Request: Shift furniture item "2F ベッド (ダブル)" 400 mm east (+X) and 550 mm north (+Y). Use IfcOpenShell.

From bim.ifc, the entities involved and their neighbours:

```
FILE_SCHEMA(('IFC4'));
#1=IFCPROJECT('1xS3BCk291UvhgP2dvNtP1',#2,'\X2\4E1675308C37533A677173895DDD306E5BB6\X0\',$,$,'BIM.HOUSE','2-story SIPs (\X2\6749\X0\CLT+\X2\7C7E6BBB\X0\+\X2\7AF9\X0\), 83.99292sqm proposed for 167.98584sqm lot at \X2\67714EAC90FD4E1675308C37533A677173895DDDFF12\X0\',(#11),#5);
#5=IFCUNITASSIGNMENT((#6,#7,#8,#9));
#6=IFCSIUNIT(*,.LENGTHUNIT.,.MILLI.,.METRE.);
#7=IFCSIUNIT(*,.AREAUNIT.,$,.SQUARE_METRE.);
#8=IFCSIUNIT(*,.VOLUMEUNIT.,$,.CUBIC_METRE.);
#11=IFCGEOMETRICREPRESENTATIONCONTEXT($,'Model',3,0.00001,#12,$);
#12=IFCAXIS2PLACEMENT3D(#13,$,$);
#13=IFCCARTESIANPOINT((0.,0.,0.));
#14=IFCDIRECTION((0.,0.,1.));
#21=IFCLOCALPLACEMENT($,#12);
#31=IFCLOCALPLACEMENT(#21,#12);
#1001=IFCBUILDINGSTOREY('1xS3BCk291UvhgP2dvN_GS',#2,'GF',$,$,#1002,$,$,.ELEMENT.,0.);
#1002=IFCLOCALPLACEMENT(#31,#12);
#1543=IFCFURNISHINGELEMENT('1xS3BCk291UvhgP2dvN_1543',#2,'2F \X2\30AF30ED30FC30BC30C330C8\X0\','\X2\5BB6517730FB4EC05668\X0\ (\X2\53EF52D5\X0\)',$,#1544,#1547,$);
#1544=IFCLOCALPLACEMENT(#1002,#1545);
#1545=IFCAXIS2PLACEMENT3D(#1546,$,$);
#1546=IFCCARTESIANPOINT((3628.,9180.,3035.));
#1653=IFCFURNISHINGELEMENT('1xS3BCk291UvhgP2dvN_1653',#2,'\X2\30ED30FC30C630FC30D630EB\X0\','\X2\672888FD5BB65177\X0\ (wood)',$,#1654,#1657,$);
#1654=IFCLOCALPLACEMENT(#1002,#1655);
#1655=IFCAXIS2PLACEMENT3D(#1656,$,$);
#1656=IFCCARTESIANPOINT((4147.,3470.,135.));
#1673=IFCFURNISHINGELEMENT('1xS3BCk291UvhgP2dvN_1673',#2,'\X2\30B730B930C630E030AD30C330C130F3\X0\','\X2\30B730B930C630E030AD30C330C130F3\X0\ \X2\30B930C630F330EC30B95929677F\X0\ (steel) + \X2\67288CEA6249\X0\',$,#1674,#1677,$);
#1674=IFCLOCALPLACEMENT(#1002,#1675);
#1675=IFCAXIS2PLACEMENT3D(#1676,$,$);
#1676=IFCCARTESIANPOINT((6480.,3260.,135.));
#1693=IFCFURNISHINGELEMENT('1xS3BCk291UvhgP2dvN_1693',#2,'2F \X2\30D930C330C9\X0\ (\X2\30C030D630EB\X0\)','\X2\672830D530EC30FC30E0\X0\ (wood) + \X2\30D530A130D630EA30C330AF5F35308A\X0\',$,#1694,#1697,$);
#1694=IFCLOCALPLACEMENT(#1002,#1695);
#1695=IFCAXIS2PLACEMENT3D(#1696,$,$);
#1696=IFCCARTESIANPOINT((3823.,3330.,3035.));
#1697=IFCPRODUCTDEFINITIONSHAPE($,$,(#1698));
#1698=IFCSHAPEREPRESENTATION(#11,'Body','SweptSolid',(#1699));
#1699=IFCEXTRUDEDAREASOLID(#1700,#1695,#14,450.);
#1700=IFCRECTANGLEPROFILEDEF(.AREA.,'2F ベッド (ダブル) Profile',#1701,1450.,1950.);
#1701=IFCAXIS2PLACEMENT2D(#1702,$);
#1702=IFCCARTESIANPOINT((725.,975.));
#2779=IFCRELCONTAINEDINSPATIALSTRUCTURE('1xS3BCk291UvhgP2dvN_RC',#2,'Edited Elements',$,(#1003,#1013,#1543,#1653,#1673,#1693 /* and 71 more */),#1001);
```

```python
import ifcopenshell
import ifcopenshell.api.geometry
import ifcopenshell.util.placement

model = ifcopenshell.open("bim.ifc")

item = model.by_id(1693)
matrix = ifcopenshell.util.placement.get_local_placement(item.ObjectPlacement)
matrix[0, 3] += 400.0
matrix[1, 3] += 550.0
ifcopenshell.api.geometry.edit_object_placement(model, product=item, matrix=matrix, is_si=False)

print(ifcopenshell.util.placement.get_local_placement(item.ObjectPlacement).round(3) + 0.0)

model.write("bim_rev.ifc")
```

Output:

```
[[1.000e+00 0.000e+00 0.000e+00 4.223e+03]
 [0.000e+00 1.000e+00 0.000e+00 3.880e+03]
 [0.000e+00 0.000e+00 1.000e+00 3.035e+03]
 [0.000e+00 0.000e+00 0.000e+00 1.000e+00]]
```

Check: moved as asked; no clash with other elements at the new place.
